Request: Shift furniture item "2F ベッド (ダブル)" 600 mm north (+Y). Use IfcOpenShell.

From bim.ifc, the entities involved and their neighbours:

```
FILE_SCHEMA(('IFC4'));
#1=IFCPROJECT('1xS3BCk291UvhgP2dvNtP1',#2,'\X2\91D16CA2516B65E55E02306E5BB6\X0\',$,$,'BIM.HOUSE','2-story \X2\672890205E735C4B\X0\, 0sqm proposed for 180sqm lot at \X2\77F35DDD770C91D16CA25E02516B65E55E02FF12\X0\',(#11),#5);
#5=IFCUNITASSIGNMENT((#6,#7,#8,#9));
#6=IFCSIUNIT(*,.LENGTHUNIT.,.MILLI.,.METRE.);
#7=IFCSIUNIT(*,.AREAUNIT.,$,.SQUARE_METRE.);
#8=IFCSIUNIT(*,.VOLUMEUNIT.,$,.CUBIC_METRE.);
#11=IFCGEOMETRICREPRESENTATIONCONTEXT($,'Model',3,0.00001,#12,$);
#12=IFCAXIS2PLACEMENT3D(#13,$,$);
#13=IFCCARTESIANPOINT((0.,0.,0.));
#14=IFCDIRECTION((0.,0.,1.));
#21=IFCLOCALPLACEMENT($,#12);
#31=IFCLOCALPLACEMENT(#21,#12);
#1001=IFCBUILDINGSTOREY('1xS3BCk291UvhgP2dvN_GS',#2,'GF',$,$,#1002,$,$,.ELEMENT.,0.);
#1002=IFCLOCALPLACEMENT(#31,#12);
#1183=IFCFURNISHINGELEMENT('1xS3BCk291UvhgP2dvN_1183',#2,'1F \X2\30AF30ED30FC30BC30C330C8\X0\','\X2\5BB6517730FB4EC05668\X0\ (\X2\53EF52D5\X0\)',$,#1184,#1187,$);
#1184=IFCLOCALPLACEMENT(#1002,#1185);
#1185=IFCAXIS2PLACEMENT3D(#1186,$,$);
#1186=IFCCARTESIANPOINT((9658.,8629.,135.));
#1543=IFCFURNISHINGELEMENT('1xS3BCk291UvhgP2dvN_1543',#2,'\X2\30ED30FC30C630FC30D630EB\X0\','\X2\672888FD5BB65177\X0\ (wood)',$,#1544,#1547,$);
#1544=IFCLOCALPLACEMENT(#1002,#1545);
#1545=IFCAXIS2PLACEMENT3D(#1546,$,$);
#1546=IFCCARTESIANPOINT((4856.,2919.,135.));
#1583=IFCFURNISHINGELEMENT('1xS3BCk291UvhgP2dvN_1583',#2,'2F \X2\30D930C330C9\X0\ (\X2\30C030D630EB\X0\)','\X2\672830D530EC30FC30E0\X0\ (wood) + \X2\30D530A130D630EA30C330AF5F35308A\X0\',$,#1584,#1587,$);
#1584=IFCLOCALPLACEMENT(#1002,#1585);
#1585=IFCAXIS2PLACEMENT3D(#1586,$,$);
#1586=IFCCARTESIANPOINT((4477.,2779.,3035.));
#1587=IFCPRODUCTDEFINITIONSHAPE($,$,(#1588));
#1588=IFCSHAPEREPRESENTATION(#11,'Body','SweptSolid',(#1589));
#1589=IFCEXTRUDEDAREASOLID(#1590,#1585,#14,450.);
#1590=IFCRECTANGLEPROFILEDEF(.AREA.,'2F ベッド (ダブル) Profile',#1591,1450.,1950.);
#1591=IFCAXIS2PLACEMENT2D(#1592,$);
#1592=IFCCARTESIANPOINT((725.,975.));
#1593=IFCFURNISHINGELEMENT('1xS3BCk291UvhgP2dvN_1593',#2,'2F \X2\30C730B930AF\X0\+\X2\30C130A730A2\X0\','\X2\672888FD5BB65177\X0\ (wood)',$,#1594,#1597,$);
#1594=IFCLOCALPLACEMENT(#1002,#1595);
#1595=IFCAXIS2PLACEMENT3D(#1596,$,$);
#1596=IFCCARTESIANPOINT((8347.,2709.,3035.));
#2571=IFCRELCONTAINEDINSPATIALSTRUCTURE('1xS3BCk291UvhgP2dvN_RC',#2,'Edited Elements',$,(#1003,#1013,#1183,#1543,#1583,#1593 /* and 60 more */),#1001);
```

```python
import ifcopenshell
import ifcopenshell.api.geometry
import ifcopenshell.util.placement
import ifcopenshell.util.unit

model = ifcopenshell.open("bim.ifc")
unit_scale = ifcopenshell.util.unit.calculate_unit_scale(model)

item = model.by_id(1583)
matrix = ifcopenshell.util.placement.get_local_placement(item.ObjectPlacement)
matrix[1, 3] += 0.6 / unit_scale
ifcopenshell.api.geometry.edit_object_placement(model, product=item, matrix=matrix, is_si=False)

print(ifcopenshell.util.placement.get_local_placement(item.ObjectPlacement).round(3) + 0.0)

model.write("bim-out.ifc")
```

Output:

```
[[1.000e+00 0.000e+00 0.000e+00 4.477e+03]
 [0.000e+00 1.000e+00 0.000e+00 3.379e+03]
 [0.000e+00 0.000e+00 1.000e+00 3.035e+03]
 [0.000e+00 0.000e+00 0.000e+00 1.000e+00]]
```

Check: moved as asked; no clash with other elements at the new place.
